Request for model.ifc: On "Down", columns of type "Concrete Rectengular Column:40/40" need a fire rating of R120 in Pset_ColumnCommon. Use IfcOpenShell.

First a look at what the model holds.

```python
import ifcopenshell
import ifcopenshell.util.element

model = ifcopenshell.open("model.ifc")
print(model.schema)
storey = next(s for s in model.by_type("IfcBuildingStorey") if s.Name == "Down")
columns = [e for e in ifcopenshell.util.element.get_decomposition(storey) if e.is_a("IfcColumn")]
seen = {}
for e in columns:
    element_type = ifcopenshell.util.element.get_type(e)
    key = (element_type.Name if element_type != e and element_type else None, ifcopenshell.util.element.get_pset(e, "Pset_ColumnCommon", "FireRating"))
    seen[key] = seen.get(key, 0) + 1
for (name, value), count in sorted(seen.items(), key=str):
    print(count, "x", name, "|", value)
```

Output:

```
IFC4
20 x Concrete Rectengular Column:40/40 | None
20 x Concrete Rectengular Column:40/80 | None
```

```python
import ifcopenshell
import ifcopenshell.api.pset
import ifcopenshell.util.element

model = ifcopenshell.open("model.ifc")

storey = next(s for s in model.by_type("IfcBuildingStorey") if s.Name == "Down")
columns = [e for e in ifcopenshell.util.element.get_decomposition(storey) if e.is_a("IfcColumn")]

count = 0
for e in columns:
    element_type = ifcopenshell.util.element.get_type(e)
    if element_type in (None, e) or element_type.Name != "Concrete Rectengular Column:40/40":
        continue
    # add_pset returns the element's existing set when there is one.
    pset = ifcopenshell.api.pset.add_pset(model, product=e, name="Pset_ColumnCommon")
    ifcopenshell.api.pset.edit_pset(model, pset=pset, properties={"FireRating": "R120"})
    count += 1

print(count, "columns updated")

model.write("model_v2.ifc")
```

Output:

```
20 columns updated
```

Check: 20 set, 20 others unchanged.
